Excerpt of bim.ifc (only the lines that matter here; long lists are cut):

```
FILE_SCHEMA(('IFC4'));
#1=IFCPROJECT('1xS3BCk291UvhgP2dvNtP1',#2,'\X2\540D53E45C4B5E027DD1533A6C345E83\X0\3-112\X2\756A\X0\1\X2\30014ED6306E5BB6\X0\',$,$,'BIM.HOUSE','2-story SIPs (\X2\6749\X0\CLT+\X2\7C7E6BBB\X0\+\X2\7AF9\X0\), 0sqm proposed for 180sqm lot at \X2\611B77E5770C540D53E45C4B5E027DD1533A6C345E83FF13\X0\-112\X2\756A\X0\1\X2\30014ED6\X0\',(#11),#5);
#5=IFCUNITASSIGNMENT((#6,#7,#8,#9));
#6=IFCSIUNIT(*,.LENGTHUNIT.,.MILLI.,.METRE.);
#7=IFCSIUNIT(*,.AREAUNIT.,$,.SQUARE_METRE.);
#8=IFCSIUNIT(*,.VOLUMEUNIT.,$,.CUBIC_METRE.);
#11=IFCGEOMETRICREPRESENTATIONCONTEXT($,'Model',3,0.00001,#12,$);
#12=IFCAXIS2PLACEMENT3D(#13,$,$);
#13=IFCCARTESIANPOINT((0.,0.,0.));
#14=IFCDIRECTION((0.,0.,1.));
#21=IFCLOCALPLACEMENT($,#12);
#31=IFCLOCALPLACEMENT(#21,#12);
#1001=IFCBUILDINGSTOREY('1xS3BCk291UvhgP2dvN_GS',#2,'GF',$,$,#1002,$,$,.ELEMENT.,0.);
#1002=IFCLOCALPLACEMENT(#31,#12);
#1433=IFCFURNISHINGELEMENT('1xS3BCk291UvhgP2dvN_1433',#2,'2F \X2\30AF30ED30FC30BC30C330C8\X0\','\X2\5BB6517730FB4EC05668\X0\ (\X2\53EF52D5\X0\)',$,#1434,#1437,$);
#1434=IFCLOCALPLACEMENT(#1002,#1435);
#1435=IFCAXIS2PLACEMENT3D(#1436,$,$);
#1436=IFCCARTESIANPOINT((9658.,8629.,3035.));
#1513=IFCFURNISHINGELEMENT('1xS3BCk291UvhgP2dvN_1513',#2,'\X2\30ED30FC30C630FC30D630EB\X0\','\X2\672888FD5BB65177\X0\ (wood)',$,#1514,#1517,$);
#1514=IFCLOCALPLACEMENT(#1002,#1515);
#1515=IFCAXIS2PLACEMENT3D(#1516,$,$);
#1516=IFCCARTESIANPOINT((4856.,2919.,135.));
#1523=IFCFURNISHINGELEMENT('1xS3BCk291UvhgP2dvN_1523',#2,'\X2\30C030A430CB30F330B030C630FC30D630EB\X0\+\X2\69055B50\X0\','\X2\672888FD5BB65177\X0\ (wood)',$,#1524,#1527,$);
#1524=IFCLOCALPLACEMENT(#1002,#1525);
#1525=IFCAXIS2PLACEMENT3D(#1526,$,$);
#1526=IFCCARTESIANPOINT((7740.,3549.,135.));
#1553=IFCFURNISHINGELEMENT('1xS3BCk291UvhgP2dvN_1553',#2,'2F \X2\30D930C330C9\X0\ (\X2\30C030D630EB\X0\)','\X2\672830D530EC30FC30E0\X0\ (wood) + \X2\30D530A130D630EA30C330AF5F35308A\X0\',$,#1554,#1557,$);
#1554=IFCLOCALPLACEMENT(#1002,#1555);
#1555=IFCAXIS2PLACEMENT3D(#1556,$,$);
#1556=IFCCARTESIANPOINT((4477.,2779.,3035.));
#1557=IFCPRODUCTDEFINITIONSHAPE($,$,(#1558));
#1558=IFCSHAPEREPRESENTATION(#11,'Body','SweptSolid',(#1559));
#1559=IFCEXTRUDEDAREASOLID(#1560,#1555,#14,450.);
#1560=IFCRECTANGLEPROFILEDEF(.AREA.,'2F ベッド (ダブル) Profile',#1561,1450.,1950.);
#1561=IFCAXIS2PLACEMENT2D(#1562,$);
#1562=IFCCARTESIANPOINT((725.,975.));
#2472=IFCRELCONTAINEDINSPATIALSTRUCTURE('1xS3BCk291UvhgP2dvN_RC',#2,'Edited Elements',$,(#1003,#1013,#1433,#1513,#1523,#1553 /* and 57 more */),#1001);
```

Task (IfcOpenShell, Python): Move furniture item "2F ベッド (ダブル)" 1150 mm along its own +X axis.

```python
import ifcopenshell
import ifcopenshell.api.geometry
import ifcopenshell.util.placement
import ifcopenshell.util.unit

model = ifcopenshell.open("bim.ifc")
unit_scale = ifcopenshell.util.unit.calculate_unit_scale(model)

item = model.by_guid("1xS3BCk291UvhgP2dvN_1553")
matrix = ifcopenshell.util.placement.get_local_placement(item.ObjectPlacement)
matrix[:3, 3] += matrix[:3, 0] * 1.15 / unit_scale
ifcopenshell.api.geometry.edit_object_placement(model, product=item, matrix=matrix, is_si=False)

print(ifcopenshell.util.placement.get_local_placement(item.ObjectPlacement).round(3) + 0.0)

model.write("bim_updated.ifc")
```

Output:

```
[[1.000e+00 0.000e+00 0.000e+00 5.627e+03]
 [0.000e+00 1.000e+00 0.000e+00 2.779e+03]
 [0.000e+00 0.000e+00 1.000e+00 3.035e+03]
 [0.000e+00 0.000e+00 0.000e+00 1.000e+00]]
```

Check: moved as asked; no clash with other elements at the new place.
